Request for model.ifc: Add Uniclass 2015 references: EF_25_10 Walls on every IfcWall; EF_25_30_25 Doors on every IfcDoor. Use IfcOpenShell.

First a look at what the model holds.

```python
import ifcopenshell

model = ifcopenshell.open("model.ifc")
print(model.schema)
print("classifications:", [c.Name for c in model.by_type("IfcClassification")])
for ifc_class in ("IfcDoor", "IfcRoof", "IfcStair", "IfcWall", "IfcWindow"):
    print(ifc_class, len(model.by_type(ifc_class)))
```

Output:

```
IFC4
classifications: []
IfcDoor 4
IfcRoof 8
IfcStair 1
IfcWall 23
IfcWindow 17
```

```python
import ifcopenshell
import ifcopenshell.api.classification

model = ifcopenshell.open("model.ifc")

system = ifcopenshell.api.classification.add_classification(model, classification="Uniclass 2015")

codes = {
    "IfcWall": ("EF_25_10", "Walls"),
    "IfcDoor": ("EF_25_30_25", "Doors"),
}
for ifc_class, (code, name) in codes.items():
    products = model.by_type(ifc_class)
    ifcopenshell.api.classification.add_reference(
        model, products=products, classification=system, identification=code, name=name
    )
    print(code, len(products))

model.write("model_rev.ifc")
```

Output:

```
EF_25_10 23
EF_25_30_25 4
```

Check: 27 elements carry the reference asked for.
